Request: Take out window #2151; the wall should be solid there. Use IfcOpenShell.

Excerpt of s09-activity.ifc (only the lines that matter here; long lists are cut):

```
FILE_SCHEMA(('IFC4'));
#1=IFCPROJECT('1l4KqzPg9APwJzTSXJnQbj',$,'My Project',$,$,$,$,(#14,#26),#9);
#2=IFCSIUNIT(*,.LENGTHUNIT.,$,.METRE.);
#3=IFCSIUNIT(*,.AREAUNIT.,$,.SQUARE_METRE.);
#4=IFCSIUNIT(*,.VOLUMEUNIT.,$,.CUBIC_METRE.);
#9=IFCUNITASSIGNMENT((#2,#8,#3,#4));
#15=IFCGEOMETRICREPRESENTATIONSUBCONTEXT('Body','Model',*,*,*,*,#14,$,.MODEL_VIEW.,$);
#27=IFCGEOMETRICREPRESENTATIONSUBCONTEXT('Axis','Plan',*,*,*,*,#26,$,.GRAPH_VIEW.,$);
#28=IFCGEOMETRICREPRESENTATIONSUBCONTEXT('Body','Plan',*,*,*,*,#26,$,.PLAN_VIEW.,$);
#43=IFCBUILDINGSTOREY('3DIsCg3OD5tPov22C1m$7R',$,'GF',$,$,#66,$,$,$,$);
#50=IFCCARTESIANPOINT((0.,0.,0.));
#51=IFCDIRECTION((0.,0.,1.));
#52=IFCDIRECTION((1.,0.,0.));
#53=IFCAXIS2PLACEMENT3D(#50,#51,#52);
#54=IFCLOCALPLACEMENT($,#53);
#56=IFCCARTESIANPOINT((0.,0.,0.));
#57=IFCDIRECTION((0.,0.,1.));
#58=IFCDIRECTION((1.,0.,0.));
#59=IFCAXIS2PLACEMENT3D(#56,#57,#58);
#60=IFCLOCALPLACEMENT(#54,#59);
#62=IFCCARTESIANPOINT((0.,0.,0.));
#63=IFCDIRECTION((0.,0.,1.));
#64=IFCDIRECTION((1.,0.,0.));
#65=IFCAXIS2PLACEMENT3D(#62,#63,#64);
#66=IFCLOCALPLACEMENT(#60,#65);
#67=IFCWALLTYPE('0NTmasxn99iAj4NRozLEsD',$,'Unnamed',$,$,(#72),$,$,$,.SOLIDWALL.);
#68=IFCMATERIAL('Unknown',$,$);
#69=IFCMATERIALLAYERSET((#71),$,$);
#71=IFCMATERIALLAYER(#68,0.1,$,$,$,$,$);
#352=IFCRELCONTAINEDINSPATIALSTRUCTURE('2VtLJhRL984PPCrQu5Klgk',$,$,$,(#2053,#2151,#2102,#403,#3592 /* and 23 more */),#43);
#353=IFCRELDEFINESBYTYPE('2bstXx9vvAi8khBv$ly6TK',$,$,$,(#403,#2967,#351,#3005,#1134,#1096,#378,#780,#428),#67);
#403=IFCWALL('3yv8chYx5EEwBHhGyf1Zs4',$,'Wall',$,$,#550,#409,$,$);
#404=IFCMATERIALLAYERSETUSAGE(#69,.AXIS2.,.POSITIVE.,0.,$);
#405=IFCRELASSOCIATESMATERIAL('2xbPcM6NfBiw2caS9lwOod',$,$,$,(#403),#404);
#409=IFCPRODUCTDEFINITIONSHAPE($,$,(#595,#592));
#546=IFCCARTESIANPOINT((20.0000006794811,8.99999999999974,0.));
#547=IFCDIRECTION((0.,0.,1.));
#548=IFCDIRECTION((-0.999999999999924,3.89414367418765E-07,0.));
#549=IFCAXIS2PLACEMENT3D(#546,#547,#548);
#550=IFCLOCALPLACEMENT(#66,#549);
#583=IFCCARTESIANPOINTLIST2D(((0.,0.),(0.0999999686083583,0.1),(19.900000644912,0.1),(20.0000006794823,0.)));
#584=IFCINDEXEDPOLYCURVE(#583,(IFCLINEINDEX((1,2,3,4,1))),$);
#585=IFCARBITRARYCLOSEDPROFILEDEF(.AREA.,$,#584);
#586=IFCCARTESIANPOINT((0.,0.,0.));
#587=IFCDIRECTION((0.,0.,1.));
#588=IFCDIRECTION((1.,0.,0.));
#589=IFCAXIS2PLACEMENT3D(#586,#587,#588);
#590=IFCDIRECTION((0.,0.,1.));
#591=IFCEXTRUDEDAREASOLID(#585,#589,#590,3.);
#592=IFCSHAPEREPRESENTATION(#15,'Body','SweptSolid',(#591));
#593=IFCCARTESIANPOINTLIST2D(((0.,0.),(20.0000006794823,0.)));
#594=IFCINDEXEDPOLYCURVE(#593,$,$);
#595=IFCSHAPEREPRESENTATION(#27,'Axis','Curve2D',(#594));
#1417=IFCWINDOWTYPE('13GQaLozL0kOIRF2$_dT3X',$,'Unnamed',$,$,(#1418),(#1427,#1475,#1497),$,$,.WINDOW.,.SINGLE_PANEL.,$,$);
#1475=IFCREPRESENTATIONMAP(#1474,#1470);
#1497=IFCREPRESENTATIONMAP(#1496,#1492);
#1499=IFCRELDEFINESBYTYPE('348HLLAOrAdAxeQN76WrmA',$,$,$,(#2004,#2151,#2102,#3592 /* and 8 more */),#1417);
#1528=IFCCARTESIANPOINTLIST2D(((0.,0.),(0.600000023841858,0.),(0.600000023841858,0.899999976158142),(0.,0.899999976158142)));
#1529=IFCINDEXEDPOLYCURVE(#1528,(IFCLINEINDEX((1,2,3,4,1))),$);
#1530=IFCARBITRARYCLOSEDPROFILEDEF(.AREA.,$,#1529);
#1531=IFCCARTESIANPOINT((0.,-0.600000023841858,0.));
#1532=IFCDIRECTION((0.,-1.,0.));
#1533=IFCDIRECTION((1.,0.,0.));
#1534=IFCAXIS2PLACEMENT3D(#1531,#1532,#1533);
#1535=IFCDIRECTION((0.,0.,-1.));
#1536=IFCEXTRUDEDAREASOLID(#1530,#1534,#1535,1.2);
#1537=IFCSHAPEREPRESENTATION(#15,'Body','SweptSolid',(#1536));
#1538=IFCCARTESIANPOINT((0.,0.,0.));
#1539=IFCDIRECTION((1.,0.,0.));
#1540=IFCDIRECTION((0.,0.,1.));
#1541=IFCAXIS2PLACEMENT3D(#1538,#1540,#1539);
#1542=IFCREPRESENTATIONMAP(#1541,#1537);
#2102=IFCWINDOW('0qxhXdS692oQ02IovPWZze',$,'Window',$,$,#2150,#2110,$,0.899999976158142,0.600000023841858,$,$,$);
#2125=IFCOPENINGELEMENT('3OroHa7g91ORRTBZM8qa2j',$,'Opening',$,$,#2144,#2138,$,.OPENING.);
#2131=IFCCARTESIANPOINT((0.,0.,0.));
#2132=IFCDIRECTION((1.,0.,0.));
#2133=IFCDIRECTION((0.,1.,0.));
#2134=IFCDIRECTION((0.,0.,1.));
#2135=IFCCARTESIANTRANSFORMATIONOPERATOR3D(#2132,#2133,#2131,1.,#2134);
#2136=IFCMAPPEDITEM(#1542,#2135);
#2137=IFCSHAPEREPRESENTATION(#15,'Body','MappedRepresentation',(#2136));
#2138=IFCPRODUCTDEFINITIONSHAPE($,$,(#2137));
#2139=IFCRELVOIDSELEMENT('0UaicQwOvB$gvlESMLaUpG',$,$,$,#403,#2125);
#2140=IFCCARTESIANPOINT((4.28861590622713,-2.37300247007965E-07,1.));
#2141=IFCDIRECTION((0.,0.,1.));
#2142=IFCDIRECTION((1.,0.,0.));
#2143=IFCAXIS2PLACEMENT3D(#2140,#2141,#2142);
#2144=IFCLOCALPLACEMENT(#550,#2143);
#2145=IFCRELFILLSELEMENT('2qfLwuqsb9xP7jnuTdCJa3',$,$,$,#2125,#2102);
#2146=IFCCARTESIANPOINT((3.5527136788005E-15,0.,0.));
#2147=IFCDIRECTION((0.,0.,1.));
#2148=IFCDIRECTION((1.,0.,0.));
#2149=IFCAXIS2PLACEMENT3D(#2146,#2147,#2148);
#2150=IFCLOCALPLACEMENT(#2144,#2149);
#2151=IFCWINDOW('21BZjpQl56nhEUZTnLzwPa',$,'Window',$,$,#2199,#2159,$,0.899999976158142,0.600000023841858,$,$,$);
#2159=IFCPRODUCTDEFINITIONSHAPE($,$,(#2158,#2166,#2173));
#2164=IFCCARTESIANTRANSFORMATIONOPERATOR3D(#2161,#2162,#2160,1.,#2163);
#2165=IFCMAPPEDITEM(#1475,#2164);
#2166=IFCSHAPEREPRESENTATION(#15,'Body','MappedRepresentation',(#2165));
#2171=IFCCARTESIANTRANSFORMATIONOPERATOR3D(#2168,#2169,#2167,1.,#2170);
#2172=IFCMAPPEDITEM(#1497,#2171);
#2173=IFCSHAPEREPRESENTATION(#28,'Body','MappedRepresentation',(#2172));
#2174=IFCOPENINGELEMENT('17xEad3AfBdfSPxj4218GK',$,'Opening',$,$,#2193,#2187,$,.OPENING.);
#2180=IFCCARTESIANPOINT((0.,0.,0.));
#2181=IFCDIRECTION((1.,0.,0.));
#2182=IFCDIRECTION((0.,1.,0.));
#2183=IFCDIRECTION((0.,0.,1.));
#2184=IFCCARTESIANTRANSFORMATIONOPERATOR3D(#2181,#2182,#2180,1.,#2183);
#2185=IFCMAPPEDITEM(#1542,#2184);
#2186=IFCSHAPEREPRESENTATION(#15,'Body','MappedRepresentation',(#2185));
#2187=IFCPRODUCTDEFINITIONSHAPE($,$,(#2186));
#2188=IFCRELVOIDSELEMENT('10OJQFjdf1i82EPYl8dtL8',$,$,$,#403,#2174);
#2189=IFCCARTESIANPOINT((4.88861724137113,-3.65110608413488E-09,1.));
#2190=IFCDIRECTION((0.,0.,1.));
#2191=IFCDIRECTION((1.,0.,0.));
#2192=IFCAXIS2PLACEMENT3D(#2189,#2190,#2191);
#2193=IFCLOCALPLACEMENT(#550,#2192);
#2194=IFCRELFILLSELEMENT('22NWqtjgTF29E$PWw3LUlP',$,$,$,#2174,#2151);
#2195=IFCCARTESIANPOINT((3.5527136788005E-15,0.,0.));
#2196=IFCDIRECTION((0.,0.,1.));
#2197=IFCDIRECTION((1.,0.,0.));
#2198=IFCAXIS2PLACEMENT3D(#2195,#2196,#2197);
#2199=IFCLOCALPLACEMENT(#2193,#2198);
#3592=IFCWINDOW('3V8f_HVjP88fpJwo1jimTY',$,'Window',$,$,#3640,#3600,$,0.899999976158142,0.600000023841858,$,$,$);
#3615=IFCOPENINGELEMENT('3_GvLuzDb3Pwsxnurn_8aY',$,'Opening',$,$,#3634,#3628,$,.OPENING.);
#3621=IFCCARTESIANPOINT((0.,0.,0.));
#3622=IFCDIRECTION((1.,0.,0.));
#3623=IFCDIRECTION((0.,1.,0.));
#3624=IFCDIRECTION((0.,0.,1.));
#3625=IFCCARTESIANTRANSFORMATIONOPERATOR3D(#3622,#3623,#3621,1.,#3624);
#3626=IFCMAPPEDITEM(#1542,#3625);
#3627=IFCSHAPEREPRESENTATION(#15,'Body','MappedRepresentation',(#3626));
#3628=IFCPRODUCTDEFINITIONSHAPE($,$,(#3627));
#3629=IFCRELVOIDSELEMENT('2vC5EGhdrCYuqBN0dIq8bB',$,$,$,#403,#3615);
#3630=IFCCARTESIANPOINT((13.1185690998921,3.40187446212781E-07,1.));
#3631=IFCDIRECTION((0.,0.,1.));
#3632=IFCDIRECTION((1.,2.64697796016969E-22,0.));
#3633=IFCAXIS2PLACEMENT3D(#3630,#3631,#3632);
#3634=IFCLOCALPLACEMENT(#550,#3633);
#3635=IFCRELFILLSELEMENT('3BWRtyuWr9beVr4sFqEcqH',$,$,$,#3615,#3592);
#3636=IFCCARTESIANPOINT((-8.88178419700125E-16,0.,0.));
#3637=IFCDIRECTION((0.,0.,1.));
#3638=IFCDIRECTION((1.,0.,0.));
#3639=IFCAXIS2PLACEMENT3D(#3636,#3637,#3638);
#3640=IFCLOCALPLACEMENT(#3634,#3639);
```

```python
import ifcopenshell
import ifcopenshell.api.feature
import ifcopenshell.api.root
import ifcopenshell.geom
import ifcopenshell.util.shape

model = ifcopenshell.open("s09-activity.ifc")
settings = ifcopenshell.geom.settings()


def volume(element):
    """Net volume in cubic metres, openings subtracted."""
    shape = ifcopenshell.geom.create_shape(settings, element)
    return ifcopenshell.util.shape.get_volume(shape.geometry)


window = model.by_guid("21BZjpQl56nhEUZTnLzwPa")
opening = window.FillsVoids[0].RelatingOpeningElement
wall = opening.VoidsElements[0].RelatingBuildingElement
before = volume(wall)

ifcopenshell.api.root.remove_product(model, product=window)
ifcopenshell.api.feature.remove_feature(model, feature=opening)

after = volume(wall)

print(f"wall volume {before:.3f} -> {after:.3f} m3")

model.write("s09-activity_edited.ifc")
```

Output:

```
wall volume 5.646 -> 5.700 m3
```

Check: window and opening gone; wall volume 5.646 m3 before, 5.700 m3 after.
